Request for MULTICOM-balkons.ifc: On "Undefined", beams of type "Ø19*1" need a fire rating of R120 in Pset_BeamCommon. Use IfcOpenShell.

First a look at what the model holds.

```python
import ifcopenshell
import ifcopenshell.util.element

model = ifcopenshell.open("MULTICOM-balkons.ifc")
print(model.schema)
storey = next(s for s in model.by_type("IfcBuildingStorey") if s.Name == "Undefined")
beams = [e for e in ifcopenshell.util.element.get_decomposition(storey) if e.is_a("IfcBeam")]
seen = {}
for e in beams:
    element_type = ifcopenshell.util.element.get_type(e)
    key = (element_type.Name if element_type != e and element_type else None, ifcopenshell.util.element.get_pset(e, "Pset_BeamCommon", "FireRating"))
    seen[key] = seen.get(key, 0) + 1
for (name, value), count in sorted(seen.items(), key=str):
    print(count, "x", name, "|", value)
```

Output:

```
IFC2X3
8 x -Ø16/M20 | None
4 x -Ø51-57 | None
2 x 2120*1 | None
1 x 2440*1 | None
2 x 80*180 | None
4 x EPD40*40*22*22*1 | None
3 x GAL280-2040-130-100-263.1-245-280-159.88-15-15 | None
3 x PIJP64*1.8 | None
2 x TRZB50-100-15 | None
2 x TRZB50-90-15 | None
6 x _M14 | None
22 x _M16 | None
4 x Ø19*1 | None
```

```python
import ifcopenshell
import ifcopenshell.api.pset
import ifcopenshell.util.element

model = ifcopenshell.open("MULTICOM-balkons.ifc")

storey = next(s for s in model.by_type("IfcBuildingStorey") if s.Name == "Undefined")
beams = [e for e in ifcopenshell.util.element.get_decomposition(storey) if e.is_a("IfcBeam")]

count = 0
for e in beams:
    element_type = ifcopenshell.util.element.get_type(e)
    if element_type in (None, e) or element_type.Name != "Ø19*1":
        continue
    # add_pset returns the element's existing set when there is one.
    pset = ifcopenshell.api.pset.add_pset(model, product=e, name="Pset_BeamCommon")
    ifcopenshell.api.pset.edit_pset(model, pset=pset, properties={"FireRating": "R120"})
    count += 1

print(count, "beams updated")

model.write("MULTICOM-balkons_rev.ifc")
```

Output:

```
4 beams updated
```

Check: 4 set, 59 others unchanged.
